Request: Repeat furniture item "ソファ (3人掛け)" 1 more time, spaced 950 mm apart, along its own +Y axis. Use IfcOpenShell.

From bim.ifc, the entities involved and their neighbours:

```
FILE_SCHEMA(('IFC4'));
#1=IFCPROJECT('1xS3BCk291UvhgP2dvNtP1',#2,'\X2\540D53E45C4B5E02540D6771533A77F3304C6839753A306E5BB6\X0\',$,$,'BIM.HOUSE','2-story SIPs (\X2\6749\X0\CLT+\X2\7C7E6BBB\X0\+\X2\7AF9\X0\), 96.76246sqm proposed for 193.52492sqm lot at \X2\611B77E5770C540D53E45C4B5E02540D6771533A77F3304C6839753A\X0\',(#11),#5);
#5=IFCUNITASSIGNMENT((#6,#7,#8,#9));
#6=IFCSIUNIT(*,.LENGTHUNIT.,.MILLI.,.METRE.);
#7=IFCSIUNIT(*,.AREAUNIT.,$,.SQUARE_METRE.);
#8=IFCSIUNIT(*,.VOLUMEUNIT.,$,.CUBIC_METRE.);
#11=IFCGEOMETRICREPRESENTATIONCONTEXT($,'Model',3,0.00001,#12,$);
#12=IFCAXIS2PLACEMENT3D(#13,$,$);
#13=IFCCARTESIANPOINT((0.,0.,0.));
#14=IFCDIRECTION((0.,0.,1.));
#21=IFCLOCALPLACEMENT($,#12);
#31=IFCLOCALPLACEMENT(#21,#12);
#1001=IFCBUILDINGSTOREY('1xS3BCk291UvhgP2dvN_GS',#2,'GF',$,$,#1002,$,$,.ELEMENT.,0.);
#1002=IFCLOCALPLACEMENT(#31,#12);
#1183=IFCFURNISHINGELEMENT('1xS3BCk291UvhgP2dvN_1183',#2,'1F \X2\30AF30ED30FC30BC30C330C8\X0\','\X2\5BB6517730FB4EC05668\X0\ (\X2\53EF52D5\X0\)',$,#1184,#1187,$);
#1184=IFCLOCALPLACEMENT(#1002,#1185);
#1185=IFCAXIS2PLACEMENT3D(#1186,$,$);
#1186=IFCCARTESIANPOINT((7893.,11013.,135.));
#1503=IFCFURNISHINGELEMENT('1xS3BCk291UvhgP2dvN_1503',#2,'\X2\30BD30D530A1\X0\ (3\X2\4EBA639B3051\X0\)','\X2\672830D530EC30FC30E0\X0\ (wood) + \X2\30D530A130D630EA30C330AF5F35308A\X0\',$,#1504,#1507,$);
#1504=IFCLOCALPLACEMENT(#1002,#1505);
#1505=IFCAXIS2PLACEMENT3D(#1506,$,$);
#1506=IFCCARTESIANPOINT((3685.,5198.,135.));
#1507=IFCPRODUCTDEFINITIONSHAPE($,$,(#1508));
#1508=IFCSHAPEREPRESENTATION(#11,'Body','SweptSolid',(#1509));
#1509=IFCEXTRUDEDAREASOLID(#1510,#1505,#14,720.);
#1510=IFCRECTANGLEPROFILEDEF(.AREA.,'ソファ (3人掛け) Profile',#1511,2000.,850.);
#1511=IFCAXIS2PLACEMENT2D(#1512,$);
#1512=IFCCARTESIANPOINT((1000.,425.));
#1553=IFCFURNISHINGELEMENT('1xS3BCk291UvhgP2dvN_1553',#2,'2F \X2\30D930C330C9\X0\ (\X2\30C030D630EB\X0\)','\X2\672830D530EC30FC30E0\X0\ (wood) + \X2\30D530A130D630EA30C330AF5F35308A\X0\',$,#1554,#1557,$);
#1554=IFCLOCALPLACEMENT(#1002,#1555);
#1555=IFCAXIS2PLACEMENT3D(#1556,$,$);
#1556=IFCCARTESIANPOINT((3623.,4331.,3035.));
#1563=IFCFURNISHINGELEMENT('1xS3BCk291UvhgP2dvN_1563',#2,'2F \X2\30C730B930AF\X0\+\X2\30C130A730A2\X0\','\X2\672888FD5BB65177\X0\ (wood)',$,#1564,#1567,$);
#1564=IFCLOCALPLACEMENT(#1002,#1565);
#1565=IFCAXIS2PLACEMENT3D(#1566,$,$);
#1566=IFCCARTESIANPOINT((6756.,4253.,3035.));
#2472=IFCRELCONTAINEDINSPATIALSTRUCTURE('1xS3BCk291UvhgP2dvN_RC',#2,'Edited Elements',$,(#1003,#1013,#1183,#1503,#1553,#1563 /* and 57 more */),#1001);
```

```python
import ifcopenshell
import ifcopenshell.api.geometry
import ifcopenshell.api.root
import ifcopenshell.util.element
import ifcopenshell.util.placement
import ifcopenshell.util.unit

model = ifcopenshell.open("bim.ifc")
unit_scale = ifcopenshell.util.unit.calculate_unit_scale(model)


def reuse_history(source, copy):
    """copy_class also copies each property set's owner history, people and application; keep the originals."""
    for rel in copy.IsDefinedBy:
        if rel.is_a("IfcRelDefinesByProperties") and (history := rel.RelatingPropertyDefinition.OwnerHistory):
            rel.RelatingPropertyDefinition.OwnerHistory = source.OwnerHistory
            ifcopenshell.util.element.remove_deep2(model, history)


source = model.by_id(1503)
base = ifcopenshell.util.placement.get_local_placement(source.ObjectPlacement)
step = base[:3, 1] * 0.95 / unit_scale

for i in range(1, 2):
    copy = ifcopenshell.api.root.copy_class(model, product=source)
    copy.Representation = ifcopenshell.util.element.copy_deep(
        model, source.Representation, exclude=["IfcGeometricRepresentationContext", "IfcRepresentationMap"]
    )
    reuse_history(source, copy)
    matrix = base.copy()
    matrix[:3, 3] += i * step
    print("added at", matrix[:3, 3].round(3) + 0.0)
    ifcopenshell.api.geometry.edit_object_placement(model, product=copy, matrix=matrix, is_si=False)

model.write("bim-out.ifc")
```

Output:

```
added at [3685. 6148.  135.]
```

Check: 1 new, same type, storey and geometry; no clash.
